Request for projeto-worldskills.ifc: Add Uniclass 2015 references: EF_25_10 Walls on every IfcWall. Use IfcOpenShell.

First a look at what the model holds.

```python
import ifcopenshell

model = ifcopenshell.open("projeto-worldskills.ifc")
print(model.schema)
print("classifications:", [c.Name for c in model.by_type("IfcClassification")])
for ifc_class in ("IfcDoor", "IfcRoof", "IfcStair", "IfcWall", "IfcWindow"):
    print(ifc_class, len(model.by_type(ifc_class)))
```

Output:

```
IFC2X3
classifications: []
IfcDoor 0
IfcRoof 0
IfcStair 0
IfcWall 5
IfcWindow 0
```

```python
import ifcopenshell
import ifcopenshell.api.classification

model = ifcopenshell.open("projeto-worldskills.ifc")

# IFC2X3 requires Source and Edition and has no link from the project to the system.
system = model.create_entity("IfcClassification", Source="NBS", Edition="2015", Name="Uniclass 2015")

codes = {
    "IfcWall": ("EF_25_10", "Walls"),
}
for ifc_class, (code, name) in codes.items():
    products = model.by_type(ifc_class)
    ifcopenshell.api.classification.add_reference(
        model, products=products, classification=system, identification=code, name=name
    )
    print(code, len(products))

model.write("projeto-worldskills_updated.ifc")
```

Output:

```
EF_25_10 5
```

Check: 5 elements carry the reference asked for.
